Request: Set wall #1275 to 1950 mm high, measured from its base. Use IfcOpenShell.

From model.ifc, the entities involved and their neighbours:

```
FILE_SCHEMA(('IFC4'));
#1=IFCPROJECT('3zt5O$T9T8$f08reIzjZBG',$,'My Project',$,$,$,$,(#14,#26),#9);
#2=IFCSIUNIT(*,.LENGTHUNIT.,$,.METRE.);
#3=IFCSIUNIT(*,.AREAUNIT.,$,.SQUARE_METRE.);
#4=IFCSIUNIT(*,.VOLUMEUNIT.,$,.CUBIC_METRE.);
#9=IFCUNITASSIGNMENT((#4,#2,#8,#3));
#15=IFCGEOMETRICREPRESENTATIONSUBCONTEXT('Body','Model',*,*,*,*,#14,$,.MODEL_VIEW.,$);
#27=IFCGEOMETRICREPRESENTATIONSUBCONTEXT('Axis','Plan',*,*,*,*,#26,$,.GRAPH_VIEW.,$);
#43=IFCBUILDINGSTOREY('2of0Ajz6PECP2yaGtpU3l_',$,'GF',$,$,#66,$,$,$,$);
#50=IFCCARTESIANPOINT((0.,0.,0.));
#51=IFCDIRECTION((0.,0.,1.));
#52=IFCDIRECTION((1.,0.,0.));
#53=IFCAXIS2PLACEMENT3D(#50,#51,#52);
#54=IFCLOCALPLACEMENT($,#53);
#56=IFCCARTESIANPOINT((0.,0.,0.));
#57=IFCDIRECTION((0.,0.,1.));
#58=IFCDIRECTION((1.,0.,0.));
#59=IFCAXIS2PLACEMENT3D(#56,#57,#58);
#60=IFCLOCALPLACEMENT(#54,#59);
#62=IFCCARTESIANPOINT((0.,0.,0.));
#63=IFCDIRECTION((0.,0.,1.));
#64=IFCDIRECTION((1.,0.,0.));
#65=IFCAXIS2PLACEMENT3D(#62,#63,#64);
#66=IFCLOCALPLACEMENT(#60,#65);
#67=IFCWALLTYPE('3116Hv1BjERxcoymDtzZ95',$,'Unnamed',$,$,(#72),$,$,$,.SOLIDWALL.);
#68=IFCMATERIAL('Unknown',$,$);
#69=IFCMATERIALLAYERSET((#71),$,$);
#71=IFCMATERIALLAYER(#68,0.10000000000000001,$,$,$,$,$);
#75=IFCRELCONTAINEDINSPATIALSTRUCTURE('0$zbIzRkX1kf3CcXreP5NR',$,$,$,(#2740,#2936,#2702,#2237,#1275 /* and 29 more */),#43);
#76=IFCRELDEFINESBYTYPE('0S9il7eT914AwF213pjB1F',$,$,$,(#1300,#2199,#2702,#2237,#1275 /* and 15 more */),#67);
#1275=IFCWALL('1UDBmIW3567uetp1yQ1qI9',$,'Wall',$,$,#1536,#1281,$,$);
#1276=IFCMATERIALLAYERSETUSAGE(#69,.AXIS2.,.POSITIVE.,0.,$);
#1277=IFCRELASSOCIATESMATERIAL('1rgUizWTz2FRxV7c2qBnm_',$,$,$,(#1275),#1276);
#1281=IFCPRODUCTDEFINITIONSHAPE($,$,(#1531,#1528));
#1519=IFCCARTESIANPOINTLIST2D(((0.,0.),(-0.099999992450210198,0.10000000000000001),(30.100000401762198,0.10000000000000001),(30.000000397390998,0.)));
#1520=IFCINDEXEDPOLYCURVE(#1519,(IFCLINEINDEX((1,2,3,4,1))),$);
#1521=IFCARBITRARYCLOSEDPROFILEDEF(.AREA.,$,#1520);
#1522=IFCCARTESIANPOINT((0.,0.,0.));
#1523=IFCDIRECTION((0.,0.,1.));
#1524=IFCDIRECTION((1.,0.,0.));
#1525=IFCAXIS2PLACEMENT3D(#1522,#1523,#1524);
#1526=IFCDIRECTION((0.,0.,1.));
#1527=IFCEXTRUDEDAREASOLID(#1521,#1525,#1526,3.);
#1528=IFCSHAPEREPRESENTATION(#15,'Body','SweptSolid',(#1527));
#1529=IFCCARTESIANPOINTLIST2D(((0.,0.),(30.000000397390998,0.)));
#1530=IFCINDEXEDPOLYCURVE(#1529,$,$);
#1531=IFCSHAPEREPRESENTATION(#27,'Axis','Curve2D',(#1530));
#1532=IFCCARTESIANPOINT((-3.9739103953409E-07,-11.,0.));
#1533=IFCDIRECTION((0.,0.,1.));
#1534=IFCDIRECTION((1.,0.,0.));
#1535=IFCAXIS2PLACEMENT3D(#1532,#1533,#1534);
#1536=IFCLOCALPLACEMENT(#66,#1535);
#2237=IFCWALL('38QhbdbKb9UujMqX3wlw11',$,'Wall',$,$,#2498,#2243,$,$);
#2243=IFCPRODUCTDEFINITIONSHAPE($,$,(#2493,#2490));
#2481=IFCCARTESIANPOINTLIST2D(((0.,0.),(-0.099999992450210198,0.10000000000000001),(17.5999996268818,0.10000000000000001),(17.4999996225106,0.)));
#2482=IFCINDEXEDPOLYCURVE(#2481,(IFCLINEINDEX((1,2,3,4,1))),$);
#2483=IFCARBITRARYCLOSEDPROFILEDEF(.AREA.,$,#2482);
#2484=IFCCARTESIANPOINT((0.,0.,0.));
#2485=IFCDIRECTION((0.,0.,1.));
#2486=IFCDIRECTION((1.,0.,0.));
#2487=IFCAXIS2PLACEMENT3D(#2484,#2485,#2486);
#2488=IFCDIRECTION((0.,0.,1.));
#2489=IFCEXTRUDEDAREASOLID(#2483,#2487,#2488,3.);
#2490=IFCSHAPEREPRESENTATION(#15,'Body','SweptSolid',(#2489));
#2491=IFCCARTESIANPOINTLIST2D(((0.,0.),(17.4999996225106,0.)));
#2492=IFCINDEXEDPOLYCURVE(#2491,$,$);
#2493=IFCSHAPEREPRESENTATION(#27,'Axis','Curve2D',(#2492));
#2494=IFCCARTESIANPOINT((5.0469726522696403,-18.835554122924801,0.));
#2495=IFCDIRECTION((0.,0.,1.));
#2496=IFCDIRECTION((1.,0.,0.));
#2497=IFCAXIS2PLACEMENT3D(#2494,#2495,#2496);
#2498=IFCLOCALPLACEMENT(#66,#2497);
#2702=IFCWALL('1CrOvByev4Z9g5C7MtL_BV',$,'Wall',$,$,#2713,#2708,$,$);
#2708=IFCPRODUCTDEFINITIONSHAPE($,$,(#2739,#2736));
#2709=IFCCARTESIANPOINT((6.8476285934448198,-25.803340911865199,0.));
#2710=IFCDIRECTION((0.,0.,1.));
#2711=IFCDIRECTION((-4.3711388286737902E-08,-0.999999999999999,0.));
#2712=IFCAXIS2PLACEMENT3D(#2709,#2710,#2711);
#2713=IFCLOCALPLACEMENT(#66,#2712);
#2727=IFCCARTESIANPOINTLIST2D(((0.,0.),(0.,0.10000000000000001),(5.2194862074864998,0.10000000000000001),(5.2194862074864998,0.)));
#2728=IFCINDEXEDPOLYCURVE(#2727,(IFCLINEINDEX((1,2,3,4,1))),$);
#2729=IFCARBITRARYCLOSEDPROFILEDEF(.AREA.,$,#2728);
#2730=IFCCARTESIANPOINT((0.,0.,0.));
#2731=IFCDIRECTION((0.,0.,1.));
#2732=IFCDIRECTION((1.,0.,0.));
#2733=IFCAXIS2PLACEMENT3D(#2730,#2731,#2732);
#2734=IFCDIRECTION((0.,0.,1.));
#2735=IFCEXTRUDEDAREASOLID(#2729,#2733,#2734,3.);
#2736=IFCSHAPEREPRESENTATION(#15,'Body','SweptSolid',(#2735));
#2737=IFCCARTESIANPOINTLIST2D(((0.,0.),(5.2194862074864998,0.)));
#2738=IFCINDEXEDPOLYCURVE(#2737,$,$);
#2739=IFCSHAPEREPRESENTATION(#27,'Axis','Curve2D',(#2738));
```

```python
import ifcopenshell
import ifcopenshell.geom
import ifcopenshell.util.representation
import ifcopenshell.util.shape

model = ifcopenshell.open("model.ifc")
settings = ifcopenshell.geom.settings()


def volume(element):
    """Net volume in cubic metres, openings subtracted."""
    shape = ifcopenshell.geom.create_shape(settings, element)
    return ifcopenshell.util.shape.get_volume(shape.geometry)


wall = model.by_id(1275)
before = volume(wall)

body = ifcopenshell.util.representation.get_representation(wall, "Model", "Body")
solid = body.Items[0]
old_height = solid.Depth
solid.Depth = 1.95
after = volume(wall)

print(f"height {old_height:g} -> {solid.Depth:g}, volume {before:.3f} -> {after:.3f} m3")

model.write("model_v2.ifc")
```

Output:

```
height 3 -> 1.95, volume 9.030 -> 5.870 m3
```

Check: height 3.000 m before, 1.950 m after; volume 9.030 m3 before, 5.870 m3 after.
